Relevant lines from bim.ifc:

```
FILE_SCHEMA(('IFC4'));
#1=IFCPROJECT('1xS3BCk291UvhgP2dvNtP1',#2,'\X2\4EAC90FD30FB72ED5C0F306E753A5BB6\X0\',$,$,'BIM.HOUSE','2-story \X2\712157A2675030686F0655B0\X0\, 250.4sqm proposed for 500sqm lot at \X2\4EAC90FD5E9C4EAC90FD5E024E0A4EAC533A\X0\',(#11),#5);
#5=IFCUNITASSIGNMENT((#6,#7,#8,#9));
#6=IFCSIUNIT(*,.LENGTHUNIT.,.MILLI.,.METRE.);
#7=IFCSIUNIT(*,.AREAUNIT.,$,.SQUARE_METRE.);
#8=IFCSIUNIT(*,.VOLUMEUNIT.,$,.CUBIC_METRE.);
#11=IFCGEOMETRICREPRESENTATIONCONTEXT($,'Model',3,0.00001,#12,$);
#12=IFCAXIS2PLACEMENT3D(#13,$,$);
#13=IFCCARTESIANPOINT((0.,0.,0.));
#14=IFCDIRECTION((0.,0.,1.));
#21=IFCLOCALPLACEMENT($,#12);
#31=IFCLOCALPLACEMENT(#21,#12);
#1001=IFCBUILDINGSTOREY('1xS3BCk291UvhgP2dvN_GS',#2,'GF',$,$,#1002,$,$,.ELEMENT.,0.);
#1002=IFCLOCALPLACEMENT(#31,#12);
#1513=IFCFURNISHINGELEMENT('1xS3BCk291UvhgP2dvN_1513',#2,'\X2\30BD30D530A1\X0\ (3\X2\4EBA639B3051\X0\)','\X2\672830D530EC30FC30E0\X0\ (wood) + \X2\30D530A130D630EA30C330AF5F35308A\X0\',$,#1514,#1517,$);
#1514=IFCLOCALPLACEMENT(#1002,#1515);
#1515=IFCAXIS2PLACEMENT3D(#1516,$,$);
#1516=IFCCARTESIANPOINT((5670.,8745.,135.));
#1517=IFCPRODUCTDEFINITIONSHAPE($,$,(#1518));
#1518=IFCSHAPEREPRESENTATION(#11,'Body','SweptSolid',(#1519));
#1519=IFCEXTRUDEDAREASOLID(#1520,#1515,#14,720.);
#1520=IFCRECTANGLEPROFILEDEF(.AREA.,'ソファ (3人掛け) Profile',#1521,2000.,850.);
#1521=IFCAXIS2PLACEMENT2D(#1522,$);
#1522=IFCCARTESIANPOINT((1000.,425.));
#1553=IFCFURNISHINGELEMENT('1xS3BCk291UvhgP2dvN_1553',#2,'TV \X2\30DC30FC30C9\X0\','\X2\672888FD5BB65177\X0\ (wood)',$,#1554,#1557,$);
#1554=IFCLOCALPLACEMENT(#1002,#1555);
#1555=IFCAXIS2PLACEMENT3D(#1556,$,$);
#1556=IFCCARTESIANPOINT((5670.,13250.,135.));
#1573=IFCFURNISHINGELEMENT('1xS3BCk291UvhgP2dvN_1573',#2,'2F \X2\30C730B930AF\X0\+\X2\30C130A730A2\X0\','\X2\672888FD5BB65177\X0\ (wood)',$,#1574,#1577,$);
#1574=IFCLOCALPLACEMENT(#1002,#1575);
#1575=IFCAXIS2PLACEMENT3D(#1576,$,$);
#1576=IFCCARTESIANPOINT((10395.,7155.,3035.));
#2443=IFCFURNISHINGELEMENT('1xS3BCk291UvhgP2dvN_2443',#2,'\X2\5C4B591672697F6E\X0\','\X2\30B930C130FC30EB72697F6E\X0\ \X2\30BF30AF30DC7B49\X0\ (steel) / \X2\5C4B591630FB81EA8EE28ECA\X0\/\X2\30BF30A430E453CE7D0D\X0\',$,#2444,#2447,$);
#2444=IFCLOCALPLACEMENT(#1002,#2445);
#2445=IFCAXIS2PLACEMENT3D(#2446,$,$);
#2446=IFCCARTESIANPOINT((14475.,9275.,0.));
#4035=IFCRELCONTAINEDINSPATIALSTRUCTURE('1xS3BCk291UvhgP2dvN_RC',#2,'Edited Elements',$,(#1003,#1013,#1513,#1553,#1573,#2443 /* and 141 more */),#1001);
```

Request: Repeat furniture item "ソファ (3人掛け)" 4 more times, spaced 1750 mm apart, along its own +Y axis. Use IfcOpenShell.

```python
import ifcopenshell
import ifcopenshell.api.geometry
import ifcopenshell.api.root
import ifcopenshell.util.element
import ifcopenshell.util.placement
import ifcopenshell.util.unit

model = ifcopenshell.open("bim.ifc")
unit_scale = ifcopenshell.util.unit.calculate_unit_scale(model)


def reuse_history(source, copy):
    """copy_class also copies each property set's owner history, people and application; keep the originals."""
    for rel in copy.IsDefinedBy:
        if rel.is_a("IfcRelDefinesByProperties") and (history := rel.RelatingPropertyDefinition.OwnerHistory):
            rel.RelatingPropertyDefinition.OwnerHistory = source.OwnerHistory
            ifcopenshell.util.element.remove_deep2(model, history)


source = model.by_guid("1xS3BCk291UvhgP2dvN_1513")
base = ifcopenshell.util.placement.get_local_placement(source.ObjectPlacement)
step = base[:3, 1] * 1.75 / unit_scale

for i in range(1, 5):
    copy = ifcopenshell.api.root.copy_class(model, product=source)
    copy.Representation = ifcopenshell.util.element.copy_deep(
        model, source.Representation, exclude=["IfcGeometricRepresentationContext", "IfcRepresentationMap"]
    )
    reuse_history(source, copy)
    matrix = base.copy()
    matrix[:3, 3] += i * step
    print("added at", matrix[:3, 3].round(3) + 0.0)
    ifcopenshell.api.geometry.edit_object_placement(model, product=copy, matrix=matrix, is_si=False)

model.write("bim-out.ifc")
```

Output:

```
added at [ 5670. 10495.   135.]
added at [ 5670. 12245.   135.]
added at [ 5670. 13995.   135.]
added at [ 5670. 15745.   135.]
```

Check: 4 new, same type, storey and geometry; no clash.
